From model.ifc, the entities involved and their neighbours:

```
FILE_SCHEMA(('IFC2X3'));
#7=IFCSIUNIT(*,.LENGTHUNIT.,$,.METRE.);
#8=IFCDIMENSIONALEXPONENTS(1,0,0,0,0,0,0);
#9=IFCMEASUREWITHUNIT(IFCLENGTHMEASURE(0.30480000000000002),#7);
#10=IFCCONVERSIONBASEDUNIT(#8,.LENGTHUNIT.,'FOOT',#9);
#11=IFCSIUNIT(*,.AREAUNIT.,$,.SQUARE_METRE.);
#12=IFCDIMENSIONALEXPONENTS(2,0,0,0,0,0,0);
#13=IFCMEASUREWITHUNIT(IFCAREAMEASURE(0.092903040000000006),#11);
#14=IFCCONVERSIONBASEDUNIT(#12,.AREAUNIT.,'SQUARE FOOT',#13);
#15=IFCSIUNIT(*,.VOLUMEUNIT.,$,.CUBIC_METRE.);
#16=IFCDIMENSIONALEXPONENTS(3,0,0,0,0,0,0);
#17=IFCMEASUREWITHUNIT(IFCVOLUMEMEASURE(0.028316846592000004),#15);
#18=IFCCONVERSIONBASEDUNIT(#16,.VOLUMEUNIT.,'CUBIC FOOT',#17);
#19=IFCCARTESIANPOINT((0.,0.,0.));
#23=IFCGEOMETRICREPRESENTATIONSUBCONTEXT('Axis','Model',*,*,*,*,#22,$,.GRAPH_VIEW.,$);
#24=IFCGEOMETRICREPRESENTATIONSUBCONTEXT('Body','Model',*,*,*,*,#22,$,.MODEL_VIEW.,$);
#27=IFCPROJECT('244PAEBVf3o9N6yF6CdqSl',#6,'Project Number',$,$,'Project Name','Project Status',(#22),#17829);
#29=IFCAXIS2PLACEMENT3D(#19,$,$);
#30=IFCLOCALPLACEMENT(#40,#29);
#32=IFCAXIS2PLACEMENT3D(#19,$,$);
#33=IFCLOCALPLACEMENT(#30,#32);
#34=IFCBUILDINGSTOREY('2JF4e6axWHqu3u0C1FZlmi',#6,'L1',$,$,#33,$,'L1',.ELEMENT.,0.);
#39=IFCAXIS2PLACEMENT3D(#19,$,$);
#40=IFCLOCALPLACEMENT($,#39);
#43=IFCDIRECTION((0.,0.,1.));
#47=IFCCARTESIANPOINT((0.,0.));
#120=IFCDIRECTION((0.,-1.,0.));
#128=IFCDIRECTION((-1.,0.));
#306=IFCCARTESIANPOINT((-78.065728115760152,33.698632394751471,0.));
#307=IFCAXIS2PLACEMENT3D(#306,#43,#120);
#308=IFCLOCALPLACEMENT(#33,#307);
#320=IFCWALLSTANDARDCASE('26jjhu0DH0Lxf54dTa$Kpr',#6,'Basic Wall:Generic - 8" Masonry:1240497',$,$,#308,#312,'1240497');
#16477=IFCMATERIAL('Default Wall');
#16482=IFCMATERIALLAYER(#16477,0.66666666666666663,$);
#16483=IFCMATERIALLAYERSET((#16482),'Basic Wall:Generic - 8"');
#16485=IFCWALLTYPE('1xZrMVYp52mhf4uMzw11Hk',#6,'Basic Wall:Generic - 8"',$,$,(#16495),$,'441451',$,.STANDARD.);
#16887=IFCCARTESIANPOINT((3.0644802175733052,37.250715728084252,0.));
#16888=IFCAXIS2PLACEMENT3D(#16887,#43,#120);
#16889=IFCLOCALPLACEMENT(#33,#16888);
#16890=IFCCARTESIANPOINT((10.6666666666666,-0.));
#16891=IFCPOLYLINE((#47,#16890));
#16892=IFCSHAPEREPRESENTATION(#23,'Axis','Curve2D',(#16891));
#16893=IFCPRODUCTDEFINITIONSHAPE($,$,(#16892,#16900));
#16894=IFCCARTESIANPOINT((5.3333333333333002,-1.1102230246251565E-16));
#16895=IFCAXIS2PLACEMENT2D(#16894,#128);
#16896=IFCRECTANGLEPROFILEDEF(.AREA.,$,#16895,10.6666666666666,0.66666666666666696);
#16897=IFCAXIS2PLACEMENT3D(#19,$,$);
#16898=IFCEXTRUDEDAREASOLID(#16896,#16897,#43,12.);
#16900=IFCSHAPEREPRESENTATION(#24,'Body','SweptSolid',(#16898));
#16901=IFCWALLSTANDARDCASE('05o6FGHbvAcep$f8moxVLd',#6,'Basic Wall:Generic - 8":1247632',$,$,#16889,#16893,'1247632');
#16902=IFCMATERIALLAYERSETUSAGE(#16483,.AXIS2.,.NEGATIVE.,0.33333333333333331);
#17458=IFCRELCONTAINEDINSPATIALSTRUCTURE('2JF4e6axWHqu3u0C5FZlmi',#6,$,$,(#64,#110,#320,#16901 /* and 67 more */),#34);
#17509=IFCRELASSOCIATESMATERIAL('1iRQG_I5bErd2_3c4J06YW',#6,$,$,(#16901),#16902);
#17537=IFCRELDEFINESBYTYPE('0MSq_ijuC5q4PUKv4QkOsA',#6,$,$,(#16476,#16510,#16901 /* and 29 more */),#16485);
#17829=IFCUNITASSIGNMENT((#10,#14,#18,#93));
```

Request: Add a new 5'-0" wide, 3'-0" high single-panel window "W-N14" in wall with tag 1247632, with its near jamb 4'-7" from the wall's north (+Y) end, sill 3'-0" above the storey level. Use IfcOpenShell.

```python
import numpy as np
import ifcopenshell
import ifcopenshell.api.feature
import ifcopenshell.api.geometry
import ifcopenshell.api.root
import ifcopenshell.api.spatial
import ifcopenshell.api.type
import ifcopenshell.geom
import ifcopenshell.util.element
import ifcopenshell.util.placement
import ifcopenshell.util.representation
import ifcopenshell.util.shape
import ifcopenshell.util.unit

model = ifcopenshell.open("model.ifc")
unit_scale = ifcopenshell.util.unit.calculate_unit_scale(model)
settings = ifcopenshell.geom.settings()


def volume(element):
    """Net volume in cubic metres, openings subtracted."""
    shape = ifcopenshell.geom.create_shape(settings, element)
    return ifcopenshell.util.shape.get_volume(shape.geometry)


wall = model.by_id(16901)
storey = ifcopenshell.util.element.get_container(wall, ifc_class="IfcBuildingStorey")
context = ifcopenshell.util.representation.get_context(model, "Model", "Body", "MODEL_VIEW")
before = volume(wall)

width, height, from_end, sill = 1.524, 0.9144, 1.397, 0.9144  # metres

# The wall runs along its own X axis, and the end named is its -X end.
wall_shape = ifcopenshell.geom.create_shape(settings, wall)
x, y, z = ifcopenshell.util.shape.get_vertices(wall_shape.geometry).T
start = x.min() + from_end
face, thickness = float(y.min()), float(y.max() - y.min())
wall_matrix = ifcopenshell.util.placement.get_local_placement(wall.ObjectPlacement)
level = ifcopenshell.util.placement.get_local_placement(storey.ObjectPlacement)[2, 3]


def in_wall(x, y):
    """Placement at x, y metres in the wall's axes, at sill height."""
    matrix = wall_matrix.copy()
    matrix[:, 3] = wall_matrix @ np.array([x / unit_scale, y / unit_scale, 0.0, 1.0])
    matrix[2, 3] = level + sill / unit_scale
    return matrix


# Opening: a box that overshoots both wall faces by 50 mm.
opening = ifcopenshell.api.root.create_entity(model, ifc_class="IfcOpeningElement")
box = ifcopenshell.api.geometry.add_wall_representation(
    model, context=context, length=width, height=height, thickness=thickness + 0.1
)
ifcopenshell.api.geometry.assign_representation(model, product=opening, representation=box)
ifcopenshell.api.geometry.edit_object_placement(model, product=opening, matrix=in_wall(start, face - 0.05), is_si=False)
ifcopenshell.api.feature.add_feature(model, feature=opening, element=wall)

window = ifcopenshell.api.root.create_entity(model, ifc_class="IfcWindow", name="W-N14")
window.OverallWidth, window.OverallHeight = width / unit_scale, height / unit_scale
body = ifcopenshell.api.geometry.add_window_representation(
    model,
    context=context,
    overall_width=window.OverallWidth,
    overall_height=window.OverallHeight,
    partition_type="SINGLE_PANEL",
)
ifcopenshell.api.geometry.assign_representation(model, product=window, representation=body)
ifcopenshell.api.spatial.assign_container(model, products=[window], relating_structure=storey)
fills = ifcopenshell.api.feature.add_filling(model, opening=opening, element=window)
fills.OwnerHistory = window.OwnerHistory  # required in IFC2X3

# IFC2X3 keeps the operation on the window style.
style = ifcopenshell.api.root.create_entity(model, ifc_class="IfcWindowStyle", name="W-N14")
style.OperationType, style.ConstructionType = "SINGLE_PANEL", "NOTDEFINED"
style.ParameterTakesPrecedence = style.Sizeable = False
ifcopenshell.api.type.assign_type(model, related_objects=[window], relating_type=style)

# Centre the window in the wall's thickness.
ifcopenshell.api.geometry.edit_object_placement(model, product=window, matrix=in_wall(start, face), is_si=False)
window_shape = ifcopenshell.geom.create_shape(settings, window)
depth = ifcopenshell.util.shape.get_vertices(window_shape.geometry)[:, 1]
offset = face + thickness / 2 - (depth.min() + depth.max()) / 2
ifcopenshell.api.geometry.edit_object_placement(model, product=window, matrix=in_wall(start, offset), is_si=False)

after = volume(wall)

print(f"wall volume {before:.3f} -> {after:.3f} m3")

model.write("model-out.ifc")
```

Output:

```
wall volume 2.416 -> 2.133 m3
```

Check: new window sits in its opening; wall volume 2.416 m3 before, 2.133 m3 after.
